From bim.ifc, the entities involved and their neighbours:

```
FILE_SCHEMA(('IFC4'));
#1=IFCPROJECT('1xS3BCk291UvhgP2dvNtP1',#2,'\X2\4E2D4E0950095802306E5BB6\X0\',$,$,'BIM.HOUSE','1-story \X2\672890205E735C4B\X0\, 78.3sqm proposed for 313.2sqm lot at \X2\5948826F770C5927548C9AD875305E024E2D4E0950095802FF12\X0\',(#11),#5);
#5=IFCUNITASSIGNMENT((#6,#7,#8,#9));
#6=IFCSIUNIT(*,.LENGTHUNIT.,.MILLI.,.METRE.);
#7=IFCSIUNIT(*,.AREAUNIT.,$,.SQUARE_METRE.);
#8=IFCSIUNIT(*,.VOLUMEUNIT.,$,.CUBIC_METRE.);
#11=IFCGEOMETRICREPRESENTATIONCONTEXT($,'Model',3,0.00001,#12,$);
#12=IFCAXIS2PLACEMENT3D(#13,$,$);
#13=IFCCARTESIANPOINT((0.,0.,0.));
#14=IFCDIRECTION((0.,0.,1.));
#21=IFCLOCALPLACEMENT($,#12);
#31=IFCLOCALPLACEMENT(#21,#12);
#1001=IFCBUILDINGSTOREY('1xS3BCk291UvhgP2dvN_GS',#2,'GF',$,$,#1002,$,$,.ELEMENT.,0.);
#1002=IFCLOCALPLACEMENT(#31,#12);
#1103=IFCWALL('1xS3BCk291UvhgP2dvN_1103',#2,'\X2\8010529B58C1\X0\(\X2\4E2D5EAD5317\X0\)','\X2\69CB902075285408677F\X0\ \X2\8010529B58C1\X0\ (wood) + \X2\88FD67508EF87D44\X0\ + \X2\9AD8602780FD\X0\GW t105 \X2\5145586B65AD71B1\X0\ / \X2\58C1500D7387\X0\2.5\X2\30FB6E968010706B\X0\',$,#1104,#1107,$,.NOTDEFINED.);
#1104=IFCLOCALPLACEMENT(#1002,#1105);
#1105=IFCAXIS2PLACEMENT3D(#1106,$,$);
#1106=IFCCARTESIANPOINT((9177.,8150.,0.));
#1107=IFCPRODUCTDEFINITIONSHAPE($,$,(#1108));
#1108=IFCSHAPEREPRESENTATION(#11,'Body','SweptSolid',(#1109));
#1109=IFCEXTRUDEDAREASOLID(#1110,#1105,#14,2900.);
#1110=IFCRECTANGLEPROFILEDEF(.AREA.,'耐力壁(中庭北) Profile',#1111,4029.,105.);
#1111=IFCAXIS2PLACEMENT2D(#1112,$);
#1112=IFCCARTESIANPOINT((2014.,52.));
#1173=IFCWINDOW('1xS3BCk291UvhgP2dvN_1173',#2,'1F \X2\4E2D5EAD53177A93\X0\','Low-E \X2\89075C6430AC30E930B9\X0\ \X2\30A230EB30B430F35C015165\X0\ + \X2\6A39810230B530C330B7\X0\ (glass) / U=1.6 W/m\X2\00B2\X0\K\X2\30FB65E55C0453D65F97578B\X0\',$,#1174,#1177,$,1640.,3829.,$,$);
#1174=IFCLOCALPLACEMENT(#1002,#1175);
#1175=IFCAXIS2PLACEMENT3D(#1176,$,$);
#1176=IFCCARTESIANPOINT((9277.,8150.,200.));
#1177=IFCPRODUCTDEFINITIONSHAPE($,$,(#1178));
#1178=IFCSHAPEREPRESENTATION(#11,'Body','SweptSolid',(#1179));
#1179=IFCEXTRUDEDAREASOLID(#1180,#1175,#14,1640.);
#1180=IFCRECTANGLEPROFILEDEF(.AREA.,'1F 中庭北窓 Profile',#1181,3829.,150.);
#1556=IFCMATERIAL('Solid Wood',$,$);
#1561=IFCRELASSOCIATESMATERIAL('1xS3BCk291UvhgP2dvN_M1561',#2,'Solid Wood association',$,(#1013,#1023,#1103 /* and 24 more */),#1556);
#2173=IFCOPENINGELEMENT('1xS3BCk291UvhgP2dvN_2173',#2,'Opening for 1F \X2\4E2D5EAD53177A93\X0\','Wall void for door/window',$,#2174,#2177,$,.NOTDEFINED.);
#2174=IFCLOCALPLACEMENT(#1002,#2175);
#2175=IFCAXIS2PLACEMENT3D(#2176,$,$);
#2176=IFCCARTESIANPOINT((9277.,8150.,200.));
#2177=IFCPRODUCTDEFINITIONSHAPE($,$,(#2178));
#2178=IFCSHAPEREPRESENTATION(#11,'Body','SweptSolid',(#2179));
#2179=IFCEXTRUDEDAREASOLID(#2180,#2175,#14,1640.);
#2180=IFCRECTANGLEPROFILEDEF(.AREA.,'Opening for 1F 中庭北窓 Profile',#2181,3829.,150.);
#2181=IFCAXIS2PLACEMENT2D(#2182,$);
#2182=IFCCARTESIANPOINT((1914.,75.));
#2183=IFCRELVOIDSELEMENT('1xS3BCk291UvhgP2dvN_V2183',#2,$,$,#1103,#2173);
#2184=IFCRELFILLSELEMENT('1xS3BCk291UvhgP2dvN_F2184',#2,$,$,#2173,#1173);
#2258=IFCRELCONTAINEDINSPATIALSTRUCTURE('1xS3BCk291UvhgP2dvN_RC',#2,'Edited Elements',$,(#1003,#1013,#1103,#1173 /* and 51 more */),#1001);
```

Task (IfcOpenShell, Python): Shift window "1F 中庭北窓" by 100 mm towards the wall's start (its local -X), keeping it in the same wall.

```python
import ifcopenshell
import ifcopenshell.api.geometry
import ifcopenshell.util.placement
import ifcopenshell.util.unit

model = ifcopenshell.open("bim.ifc")
unit_scale = ifcopenshell.util.unit.calculate_unit_scale(model)

window = model.by_guid("1xS3BCk291UvhgP2dvN_1173")
opening = window.FillsVoids[0].RelatingOpeningElement
wall = opening.VoidsElements[0].RelatingBuildingElement

wall_matrix = ifcopenshell.util.placement.get_local_placement(wall.ObjectPlacement)
shift = wall_matrix[:3, 0] * -0.1 / unit_scale
before = ifcopenshell.util.placement.get_local_placement(window.ObjectPlacement)[:3, 3].copy()

# The window is not placed relative to its opening, so move both.
for product in (opening, window):
    matrix = ifcopenshell.util.placement.get_local_placement(product.ObjectPlacement)
    matrix[:3, 3] += shift
    ifcopenshell.api.geometry.edit_object_placement(model, product=product, matrix=matrix, is_si=False)

after = ifcopenshell.util.placement.get_local_placement(window.ObjectPlacement)[:3, 3]
print("window moved by", (after - before).round(3) + 0.0)

model.write("bim_updated.ifc")
```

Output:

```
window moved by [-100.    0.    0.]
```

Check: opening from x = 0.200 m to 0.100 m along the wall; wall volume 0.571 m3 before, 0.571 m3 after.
